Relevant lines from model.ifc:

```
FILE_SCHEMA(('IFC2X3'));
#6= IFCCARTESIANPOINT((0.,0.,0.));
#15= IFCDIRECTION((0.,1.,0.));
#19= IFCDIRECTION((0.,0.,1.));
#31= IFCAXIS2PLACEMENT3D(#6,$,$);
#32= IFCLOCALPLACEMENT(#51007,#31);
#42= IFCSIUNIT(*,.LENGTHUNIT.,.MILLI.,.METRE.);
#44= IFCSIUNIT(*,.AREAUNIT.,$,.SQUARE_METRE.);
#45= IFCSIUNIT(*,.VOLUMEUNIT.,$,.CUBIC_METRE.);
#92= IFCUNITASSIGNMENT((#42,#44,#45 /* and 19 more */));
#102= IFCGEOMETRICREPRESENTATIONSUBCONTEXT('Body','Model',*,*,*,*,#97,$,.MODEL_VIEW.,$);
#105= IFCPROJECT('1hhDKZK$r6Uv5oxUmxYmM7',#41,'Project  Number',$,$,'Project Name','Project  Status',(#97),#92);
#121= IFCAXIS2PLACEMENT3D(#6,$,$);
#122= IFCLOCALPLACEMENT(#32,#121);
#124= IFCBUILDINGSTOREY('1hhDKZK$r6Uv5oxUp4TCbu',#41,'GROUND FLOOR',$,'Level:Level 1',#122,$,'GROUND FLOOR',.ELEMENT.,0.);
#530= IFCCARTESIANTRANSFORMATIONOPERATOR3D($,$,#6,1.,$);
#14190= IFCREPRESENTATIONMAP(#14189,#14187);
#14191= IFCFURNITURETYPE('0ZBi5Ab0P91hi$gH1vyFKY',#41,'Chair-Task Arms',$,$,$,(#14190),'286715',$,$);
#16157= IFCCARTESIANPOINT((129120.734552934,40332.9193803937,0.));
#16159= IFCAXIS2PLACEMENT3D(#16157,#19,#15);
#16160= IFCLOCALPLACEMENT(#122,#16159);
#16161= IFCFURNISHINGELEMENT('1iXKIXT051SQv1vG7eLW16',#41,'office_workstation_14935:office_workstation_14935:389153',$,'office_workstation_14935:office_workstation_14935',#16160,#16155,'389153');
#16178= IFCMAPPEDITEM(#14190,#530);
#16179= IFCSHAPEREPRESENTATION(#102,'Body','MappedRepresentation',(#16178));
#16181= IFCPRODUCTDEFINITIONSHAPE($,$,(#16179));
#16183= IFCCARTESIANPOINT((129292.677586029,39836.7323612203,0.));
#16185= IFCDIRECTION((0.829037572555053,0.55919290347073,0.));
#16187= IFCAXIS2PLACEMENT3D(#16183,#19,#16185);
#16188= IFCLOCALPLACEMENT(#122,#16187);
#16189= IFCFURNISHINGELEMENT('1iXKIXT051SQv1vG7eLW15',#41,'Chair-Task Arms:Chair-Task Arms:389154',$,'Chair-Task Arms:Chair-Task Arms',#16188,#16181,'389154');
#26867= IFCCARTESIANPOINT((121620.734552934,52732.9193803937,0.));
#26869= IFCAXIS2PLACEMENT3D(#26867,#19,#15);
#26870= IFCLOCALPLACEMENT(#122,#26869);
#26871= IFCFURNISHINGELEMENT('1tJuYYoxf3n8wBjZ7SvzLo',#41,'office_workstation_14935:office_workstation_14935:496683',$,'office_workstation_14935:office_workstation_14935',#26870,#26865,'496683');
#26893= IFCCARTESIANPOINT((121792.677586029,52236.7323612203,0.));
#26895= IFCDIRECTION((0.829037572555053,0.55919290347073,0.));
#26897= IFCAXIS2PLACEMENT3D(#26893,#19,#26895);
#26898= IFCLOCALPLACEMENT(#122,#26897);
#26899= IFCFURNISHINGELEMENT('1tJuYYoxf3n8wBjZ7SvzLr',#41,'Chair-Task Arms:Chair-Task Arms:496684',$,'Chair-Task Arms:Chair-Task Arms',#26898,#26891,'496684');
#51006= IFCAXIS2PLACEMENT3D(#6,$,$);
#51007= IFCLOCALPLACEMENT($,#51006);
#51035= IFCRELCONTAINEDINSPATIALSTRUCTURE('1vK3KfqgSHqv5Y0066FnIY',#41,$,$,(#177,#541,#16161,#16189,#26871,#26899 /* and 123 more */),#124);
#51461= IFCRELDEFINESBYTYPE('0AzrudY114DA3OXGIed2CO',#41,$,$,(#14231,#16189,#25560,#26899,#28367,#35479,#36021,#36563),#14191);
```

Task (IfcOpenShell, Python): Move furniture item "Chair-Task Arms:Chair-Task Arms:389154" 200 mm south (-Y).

```python
import ifcopenshell
import ifcopenshell.api.geometry
import ifcopenshell.util.placement

model = ifcopenshell.open("model.ifc")

item = model.by_id(16189)
matrix = ifcopenshell.util.placement.get_local_placement(item.ObjectPlacement)
matrix[1, 3] -= 200.0
ifcopenshell.api.geometry.edit_object_placement(model, product=item, matrix=matrix, is_si=False)

print(ifcopenshell.util.placement.get_local_placement(item.ObjectPlacement).round(3) + 0.0)

model.write("model_v2.ifc")
```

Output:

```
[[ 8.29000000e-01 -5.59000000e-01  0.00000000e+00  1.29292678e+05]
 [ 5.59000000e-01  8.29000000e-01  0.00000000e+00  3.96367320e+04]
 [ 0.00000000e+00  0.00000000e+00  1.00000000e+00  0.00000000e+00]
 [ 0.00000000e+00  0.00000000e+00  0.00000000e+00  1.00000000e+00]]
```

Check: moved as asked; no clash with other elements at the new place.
